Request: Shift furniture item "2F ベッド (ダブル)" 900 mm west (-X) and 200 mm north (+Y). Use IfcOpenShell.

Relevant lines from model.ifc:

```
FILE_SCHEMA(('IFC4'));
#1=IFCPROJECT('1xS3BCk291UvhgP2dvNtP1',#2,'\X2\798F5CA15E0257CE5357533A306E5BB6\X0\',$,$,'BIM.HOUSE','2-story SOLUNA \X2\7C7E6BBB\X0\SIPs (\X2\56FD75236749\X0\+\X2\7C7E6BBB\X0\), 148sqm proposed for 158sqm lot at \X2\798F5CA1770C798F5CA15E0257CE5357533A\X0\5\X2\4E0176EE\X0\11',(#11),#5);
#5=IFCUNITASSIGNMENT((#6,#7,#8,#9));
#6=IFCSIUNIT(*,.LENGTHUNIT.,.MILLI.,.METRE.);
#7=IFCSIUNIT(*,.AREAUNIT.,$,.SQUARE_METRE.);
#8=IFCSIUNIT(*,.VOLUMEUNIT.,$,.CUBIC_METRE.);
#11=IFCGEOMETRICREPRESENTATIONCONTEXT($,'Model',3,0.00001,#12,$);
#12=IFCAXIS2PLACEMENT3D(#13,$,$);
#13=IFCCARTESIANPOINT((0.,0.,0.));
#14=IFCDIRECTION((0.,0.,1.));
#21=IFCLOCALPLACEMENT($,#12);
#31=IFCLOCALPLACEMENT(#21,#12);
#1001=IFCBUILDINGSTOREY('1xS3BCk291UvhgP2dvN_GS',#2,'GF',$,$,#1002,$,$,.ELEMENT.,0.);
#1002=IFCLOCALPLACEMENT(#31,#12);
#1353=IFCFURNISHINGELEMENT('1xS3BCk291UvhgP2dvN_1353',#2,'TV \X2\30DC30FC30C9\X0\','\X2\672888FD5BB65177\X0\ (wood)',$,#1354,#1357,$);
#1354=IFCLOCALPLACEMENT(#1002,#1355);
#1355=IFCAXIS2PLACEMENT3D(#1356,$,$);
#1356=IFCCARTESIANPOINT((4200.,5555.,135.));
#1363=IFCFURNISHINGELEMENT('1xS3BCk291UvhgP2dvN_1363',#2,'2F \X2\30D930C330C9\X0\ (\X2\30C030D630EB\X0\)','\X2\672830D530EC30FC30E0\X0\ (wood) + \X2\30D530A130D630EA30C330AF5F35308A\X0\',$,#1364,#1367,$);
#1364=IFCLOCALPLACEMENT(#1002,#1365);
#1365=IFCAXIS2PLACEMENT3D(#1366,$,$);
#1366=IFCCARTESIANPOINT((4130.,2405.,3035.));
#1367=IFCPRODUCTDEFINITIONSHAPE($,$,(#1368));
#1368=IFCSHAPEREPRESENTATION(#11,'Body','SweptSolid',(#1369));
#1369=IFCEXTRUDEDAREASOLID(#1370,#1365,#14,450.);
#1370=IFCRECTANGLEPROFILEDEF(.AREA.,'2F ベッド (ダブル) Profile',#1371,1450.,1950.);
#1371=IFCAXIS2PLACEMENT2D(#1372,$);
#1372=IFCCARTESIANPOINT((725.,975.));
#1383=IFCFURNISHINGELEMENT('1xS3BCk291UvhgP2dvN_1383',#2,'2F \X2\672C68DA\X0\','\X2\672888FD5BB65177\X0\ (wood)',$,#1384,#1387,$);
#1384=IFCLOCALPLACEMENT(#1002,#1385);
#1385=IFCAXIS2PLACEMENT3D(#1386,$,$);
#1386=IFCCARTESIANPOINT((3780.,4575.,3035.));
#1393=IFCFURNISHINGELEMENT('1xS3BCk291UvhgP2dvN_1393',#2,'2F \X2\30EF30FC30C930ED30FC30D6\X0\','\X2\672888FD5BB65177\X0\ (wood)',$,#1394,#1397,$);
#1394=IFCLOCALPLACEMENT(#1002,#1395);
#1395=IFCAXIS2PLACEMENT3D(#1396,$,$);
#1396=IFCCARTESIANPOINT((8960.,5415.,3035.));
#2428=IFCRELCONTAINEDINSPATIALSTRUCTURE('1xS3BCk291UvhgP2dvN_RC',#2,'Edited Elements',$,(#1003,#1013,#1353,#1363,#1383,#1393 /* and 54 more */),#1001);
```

```python
import ifcopenshell
import ifcopenshell.api.geometry
import ifcopenshell.util.placement
import ifcopenshell.util.unit

model = ifcopenshell.open("model.ifc")
unit_scale = ifcopenshell.util.unit.calculate_unit_scale(model)

item = model.by_id(1363)
matrix = ifcopenshell.util.placement.get_local_placement(item.ObjectPlacement)
matrix[0, 3] -= 0.9 / unit_scale
matrix[1, 3] += 0.2 / unit_scale
ifcopenshell.api.geometry.edit_object_placement(model, product=item, matrix=matrix, is_si=False)

print(ifcopenshell.util.placement.get_local_placement(item.ObjectPlacement).round(3) + 0.0)

model.write("model-out.ifc")
```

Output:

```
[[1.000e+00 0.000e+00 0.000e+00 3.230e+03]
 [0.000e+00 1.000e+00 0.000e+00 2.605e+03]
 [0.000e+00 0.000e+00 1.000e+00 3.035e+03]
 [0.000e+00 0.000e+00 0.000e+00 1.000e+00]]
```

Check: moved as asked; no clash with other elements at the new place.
